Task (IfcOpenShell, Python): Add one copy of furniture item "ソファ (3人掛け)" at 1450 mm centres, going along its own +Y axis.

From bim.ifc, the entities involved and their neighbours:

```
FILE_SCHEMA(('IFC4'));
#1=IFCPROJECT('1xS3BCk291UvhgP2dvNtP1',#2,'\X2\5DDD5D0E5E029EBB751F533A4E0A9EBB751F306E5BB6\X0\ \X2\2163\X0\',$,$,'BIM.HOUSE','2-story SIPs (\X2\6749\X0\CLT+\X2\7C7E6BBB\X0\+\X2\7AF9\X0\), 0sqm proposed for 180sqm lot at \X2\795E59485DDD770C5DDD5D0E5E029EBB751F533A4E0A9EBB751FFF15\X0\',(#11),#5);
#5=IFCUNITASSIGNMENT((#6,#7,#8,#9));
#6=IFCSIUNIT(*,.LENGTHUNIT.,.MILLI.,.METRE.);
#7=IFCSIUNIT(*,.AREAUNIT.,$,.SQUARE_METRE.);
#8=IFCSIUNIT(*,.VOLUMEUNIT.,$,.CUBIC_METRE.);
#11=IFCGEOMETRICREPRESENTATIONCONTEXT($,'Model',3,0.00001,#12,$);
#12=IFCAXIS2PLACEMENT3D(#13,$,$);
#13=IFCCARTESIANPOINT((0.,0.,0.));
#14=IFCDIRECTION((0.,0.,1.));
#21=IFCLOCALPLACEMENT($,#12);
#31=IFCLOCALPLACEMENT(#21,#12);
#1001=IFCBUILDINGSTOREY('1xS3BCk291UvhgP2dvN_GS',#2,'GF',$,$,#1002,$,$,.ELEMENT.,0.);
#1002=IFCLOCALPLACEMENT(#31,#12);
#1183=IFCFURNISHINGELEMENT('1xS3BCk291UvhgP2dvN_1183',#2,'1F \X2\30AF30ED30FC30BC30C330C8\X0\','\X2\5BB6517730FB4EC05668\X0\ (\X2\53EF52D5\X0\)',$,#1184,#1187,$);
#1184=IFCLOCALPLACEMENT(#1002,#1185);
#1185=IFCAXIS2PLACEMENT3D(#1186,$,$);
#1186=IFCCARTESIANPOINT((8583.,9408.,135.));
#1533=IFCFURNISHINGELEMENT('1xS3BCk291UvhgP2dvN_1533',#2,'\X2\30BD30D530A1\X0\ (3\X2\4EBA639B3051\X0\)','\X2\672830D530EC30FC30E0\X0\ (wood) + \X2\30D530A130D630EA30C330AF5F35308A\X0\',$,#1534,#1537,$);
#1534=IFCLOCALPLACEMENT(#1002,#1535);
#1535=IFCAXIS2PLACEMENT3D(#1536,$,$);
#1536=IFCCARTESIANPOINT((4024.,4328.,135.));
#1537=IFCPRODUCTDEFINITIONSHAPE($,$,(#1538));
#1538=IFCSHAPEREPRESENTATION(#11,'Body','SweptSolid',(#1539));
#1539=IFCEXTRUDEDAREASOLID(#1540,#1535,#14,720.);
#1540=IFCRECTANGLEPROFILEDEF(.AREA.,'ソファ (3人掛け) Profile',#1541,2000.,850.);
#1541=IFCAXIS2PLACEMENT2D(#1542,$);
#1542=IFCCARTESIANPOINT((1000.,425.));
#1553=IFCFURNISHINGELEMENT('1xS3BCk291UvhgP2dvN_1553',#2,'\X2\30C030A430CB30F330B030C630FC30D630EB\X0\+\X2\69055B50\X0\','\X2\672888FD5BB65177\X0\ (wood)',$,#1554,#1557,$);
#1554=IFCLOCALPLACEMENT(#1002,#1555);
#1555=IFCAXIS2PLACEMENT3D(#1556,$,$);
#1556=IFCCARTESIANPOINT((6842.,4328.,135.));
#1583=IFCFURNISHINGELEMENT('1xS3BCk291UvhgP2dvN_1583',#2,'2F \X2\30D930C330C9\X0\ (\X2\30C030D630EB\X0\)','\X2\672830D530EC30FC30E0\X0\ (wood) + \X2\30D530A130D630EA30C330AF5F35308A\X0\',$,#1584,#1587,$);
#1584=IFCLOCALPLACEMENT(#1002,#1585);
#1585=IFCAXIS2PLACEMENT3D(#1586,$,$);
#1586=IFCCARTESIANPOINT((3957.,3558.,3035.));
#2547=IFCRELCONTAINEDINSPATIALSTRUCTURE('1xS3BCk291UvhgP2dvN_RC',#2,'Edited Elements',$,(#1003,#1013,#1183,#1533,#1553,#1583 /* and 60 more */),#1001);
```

```python
import ifcopenshell
import ifcopenshell.api.geometry
import ifcopenshell.api.root
import ifcopenshell.util.element
import ifcopenshell.util.placement

model = ifcopenshell.open("bim.ifc")


def reuse_history(source, copy):
    """copy_class also copies each property set's owner history, people and application; keep the originals."""
    for rel in copy.IsDefinedBy:
        if rel.is_a("IfcRelDefinesByProperties") and (history := rel.RelatingPropertyDefinition.OwnerHistory):
            rel.RelatingPropertyDefinition.OwnerHistory = source.OwnerHistory
            ifcopenshell.util.element.remove_deep2(model, history)


source = model.by_id(1533)
base = ifcopenshell.util.placement.get_local_placement(source.ObjectPlacement)
step = base[:3, 1] * 1450.0

for i in range(1, 2):
    copy = ifcopenshell.api.root.copy_class(model, product=source)
    copy.Representation = ifcopenshell.util.element.copy_deep(
        model, source.Representation, exclude=["IfcGeometricRepresentationContext", "IfcRepresentationMap"]
    )
    reuse_history(source, copy)
    matrix = base.copy()
    matrix[:3, 3] += i * step
    print("added at", matrix[:3, 3].round(3) + 0.0)
    ifcopenshell.api.geometry.edit_object_placement(model, product=copy, matrix=matrix, is_si=False)

model.write("bim_rev.ifc")
```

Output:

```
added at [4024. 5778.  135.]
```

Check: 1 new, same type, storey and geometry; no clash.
